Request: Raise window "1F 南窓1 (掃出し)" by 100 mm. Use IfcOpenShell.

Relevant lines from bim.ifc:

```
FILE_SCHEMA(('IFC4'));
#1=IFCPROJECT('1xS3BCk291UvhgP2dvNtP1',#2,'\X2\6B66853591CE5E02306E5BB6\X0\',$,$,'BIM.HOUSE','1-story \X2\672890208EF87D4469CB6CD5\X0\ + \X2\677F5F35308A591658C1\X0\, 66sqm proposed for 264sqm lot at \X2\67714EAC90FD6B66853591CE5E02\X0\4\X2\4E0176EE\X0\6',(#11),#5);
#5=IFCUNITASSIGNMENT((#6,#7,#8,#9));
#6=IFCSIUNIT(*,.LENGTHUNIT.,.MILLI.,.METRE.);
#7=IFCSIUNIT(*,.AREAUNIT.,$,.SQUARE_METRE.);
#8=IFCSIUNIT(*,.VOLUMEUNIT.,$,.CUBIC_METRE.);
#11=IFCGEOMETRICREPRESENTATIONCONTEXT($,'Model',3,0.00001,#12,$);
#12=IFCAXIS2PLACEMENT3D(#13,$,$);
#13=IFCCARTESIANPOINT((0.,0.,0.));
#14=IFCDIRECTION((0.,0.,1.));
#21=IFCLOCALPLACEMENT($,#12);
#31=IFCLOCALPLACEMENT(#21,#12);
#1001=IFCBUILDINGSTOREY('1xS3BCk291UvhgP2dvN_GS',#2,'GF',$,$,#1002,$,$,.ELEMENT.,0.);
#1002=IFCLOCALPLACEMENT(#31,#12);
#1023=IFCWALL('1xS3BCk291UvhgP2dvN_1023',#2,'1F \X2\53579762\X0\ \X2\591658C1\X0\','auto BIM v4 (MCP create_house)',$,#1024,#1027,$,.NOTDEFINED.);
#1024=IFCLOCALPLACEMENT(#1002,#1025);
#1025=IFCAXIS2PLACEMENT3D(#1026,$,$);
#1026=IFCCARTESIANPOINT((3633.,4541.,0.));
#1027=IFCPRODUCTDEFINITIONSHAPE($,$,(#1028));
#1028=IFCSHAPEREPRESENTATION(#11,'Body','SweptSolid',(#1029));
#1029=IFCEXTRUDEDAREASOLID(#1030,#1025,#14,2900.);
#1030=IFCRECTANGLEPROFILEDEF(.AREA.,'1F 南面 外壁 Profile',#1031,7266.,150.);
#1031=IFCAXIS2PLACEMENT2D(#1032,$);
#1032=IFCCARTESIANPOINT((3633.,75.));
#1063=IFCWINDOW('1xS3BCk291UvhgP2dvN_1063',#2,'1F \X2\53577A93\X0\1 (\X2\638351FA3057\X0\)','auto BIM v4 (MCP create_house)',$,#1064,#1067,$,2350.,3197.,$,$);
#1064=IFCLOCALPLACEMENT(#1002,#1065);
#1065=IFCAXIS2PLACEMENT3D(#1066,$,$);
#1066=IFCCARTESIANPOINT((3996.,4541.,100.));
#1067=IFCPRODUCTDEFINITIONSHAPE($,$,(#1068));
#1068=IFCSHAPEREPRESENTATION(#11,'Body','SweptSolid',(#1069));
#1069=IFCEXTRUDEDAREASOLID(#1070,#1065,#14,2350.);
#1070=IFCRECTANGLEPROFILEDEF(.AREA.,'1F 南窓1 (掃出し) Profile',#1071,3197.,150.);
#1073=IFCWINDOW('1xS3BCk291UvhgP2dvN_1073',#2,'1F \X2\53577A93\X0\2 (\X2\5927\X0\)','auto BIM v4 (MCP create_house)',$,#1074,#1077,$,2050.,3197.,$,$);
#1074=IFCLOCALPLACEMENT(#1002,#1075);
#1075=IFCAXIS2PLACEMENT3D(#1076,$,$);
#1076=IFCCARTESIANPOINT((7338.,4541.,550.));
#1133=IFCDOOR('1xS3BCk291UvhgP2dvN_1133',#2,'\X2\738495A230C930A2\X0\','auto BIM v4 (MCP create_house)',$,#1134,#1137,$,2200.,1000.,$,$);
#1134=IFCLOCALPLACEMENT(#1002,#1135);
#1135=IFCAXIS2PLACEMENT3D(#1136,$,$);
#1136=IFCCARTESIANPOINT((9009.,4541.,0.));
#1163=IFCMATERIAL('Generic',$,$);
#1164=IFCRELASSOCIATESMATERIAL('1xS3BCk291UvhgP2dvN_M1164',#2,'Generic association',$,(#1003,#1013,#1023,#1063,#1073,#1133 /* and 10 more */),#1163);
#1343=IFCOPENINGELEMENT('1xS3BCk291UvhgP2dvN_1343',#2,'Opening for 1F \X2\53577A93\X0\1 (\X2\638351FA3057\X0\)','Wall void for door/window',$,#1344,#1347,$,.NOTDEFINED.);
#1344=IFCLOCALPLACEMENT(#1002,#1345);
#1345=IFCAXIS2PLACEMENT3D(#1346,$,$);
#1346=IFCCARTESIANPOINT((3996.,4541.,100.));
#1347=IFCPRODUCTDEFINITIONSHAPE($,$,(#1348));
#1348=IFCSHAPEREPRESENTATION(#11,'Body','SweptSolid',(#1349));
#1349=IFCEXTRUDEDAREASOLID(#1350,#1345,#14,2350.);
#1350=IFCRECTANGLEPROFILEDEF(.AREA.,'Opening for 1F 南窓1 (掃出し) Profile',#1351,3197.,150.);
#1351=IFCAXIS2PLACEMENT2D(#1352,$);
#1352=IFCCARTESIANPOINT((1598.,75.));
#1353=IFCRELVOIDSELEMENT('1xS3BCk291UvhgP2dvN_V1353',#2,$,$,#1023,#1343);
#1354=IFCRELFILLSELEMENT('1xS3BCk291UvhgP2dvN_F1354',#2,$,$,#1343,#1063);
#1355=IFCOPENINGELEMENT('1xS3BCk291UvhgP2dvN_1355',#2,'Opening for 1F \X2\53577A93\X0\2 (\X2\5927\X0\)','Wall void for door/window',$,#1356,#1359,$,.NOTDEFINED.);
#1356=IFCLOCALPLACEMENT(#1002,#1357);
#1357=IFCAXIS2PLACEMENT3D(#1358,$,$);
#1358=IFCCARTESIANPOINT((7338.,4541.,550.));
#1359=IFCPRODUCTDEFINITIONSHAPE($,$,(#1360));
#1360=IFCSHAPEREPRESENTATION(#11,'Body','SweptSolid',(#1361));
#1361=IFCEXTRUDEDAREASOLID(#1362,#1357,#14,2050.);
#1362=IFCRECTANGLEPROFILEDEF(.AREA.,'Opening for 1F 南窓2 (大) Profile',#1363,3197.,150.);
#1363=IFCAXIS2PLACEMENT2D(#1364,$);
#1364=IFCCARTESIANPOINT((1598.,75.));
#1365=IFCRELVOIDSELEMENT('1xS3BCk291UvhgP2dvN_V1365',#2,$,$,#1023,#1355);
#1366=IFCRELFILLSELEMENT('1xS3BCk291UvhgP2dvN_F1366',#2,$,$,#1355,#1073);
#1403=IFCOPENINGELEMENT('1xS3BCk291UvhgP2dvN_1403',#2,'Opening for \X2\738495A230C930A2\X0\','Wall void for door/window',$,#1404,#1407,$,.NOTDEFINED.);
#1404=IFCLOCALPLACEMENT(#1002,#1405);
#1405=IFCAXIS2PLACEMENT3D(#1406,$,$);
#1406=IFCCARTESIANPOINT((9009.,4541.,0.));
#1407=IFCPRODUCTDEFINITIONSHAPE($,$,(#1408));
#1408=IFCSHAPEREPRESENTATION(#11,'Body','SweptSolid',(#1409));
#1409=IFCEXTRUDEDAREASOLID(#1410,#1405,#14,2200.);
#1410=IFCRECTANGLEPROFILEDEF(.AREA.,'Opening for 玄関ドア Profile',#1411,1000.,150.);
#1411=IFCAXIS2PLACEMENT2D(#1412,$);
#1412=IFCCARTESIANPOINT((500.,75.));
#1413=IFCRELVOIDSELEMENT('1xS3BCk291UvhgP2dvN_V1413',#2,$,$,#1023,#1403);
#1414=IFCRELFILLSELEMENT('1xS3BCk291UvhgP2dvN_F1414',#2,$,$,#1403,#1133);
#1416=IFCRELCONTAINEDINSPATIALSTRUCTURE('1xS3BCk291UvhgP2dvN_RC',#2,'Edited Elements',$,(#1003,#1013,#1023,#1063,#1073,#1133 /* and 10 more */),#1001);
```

```python
import numpy as np
import ifcopenshell
import ifcopenshell.api.geometry
import ifcopenshell.util.placement
import ifcopenshell.util.unit

model = ifcopenshell.open("bim.ifc")
unit_scale = ifcopenshell.util.unit.calculate_unit_scale(model)

window = model.by_id(1063)
opening = window.FillsVoids[0].RelatingOpeningElement
dz = 0.1 / unit_scale

shift = np.array([0.0, 0.0, dz])
# The window is not placed relative to its opening, so move both.
for product in (opening, window):
    matrix = ifcopenshell.util.placement.get_local_placement(product.ObjectPlacement)
    matrix[:3, 3] += shift
    ifcopenshell.api.geometry.edit_object_placement(model, product=product, matrix=matrix, is_si=False)

print(f"moved by {dz * unit_scale:+.3f} m")

model.write("bim_v2.ifc")
```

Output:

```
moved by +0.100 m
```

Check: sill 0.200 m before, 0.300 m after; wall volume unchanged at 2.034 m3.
